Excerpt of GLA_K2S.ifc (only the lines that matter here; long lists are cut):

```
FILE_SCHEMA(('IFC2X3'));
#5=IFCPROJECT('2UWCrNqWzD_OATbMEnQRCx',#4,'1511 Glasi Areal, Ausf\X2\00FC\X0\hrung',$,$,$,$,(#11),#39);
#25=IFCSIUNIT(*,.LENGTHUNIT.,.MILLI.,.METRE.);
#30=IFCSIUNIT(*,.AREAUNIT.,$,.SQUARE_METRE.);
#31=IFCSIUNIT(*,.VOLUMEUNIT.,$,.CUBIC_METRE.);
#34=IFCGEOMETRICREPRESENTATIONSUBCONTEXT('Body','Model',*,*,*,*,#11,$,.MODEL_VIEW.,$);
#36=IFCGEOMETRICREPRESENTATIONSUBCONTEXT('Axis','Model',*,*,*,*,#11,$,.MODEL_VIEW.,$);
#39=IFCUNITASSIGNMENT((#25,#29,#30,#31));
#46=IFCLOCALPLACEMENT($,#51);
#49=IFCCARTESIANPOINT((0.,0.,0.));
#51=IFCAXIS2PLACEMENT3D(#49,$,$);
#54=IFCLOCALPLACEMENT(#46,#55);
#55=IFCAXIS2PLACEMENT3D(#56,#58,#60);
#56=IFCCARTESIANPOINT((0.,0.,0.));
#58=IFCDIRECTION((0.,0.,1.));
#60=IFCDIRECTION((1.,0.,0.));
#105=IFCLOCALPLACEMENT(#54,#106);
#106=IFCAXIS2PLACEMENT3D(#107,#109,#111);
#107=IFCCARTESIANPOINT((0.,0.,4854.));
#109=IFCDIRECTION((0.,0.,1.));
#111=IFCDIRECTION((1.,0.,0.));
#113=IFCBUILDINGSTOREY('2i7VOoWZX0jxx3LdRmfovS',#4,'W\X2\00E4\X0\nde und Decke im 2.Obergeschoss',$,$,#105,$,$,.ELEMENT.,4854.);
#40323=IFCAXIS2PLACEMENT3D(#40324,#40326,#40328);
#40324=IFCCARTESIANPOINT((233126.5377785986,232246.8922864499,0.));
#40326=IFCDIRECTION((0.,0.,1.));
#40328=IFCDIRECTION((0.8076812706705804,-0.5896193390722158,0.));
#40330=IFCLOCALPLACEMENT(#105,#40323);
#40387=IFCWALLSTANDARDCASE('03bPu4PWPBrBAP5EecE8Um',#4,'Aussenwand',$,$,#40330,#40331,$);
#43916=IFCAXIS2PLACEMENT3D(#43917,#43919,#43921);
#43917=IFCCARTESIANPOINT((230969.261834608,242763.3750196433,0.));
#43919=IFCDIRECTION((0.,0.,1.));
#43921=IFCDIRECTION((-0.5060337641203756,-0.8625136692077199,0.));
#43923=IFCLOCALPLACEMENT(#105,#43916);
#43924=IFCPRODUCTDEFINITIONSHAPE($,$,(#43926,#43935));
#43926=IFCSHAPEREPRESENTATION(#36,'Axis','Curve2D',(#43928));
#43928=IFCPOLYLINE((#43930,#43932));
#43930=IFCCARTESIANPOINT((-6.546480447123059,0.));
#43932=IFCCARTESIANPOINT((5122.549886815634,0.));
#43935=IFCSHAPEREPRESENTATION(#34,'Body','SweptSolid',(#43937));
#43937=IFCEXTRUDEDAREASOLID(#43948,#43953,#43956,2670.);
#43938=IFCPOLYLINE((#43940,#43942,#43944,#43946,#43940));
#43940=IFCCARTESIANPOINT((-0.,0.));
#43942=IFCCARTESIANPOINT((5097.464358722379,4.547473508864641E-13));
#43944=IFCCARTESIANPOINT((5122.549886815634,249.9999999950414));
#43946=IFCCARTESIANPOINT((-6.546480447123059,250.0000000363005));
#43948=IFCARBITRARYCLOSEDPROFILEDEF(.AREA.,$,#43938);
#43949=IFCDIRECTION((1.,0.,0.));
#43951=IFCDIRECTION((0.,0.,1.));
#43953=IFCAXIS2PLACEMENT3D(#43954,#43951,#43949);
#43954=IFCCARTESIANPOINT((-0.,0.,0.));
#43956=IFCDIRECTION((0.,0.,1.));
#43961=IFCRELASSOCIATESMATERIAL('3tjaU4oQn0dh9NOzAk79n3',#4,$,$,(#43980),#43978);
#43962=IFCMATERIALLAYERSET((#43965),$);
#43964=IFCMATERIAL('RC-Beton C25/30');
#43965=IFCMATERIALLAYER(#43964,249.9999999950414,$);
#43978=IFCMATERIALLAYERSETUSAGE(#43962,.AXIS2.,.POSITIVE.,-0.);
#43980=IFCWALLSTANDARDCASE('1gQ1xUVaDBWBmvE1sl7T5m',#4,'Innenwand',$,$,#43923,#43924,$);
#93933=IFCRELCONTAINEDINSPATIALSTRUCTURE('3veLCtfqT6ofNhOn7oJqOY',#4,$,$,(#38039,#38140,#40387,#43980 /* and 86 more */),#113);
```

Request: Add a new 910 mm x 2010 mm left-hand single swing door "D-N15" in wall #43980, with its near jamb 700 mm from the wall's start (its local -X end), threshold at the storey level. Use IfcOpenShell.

```python
import numpy as np
import ifcopenshell
import ifcopenshell.api.feature
import ifcopenshell.api.geometry
import ifcopenshell.api.root
import ifcopenshell.api.spatial
import ifcopenshell.api.type
import ifcopenshell.geom
import ifcopenshell.util.element
import ifcopenshell.util.placement
import ifcopenshell.util.representation
import ifcopenshell.util.shape
import ifcopenshell.util.unit

model = ifcopenshell.open("GLA_K2S.ifc")
unit_scale = ifcopenshell.util.unit.calculate_unit_scale(model)
settings = ifcopenshell.geom.settings()


def volume(element):
    """Net volume in cubic metres, openings subtracted."""
    shape = ifcopenshell.geom.create_shape(settings, element)
    return ifcopenshell.util.shape.get_volume(shape.geometry)


wall = model.by_id(43980)
storey = ifcopenshell.util.element.get_container(wall, ifc_class="IfcBuildingStorey")
context = ifcopenshell.util.representation.get_context(model, "Model", "Body", "MODEL_VIEW")
before = volume(wall)

width, height, from_end, sill = 0.91, 2.01, 0.7, 0.0  # metres

# The wall runs along its own X axis, and the end named is its -X end.
wall_shape = ifcopenshell.geom.create_shape(settings, wall)
x, y, z = ifcopenshell.util.shape.get_vertices(wall_shape.geometry).T
start = x.min() + from_end
face, thickness = float(y.min()), float(y.max() - y.min())
wall_matrix = ifcopenshell.util.placement.get_local_placement(wall.ObjectPlacement)
level = ifcopenshell.util.placement.get_local_placement(storey.ObjectPlacement)[2, 3]


def in_wall(x, y):
    """Placement at x, y metres in the wall's axes, at sill height."""
    matrix = wall_matrix.copy()
    matrix[:, 3] = wall_matrix @ np.array([x / unit_scale, y / unit_scale, 0.0, 1.0])
    matrix[2, 3] = level + sill / unit_scale
    return matrix


# Opening: a box that overshoots both wall faces by 50 mm.
opening = ifcopenshell.api.root.create_entity(model, ifc_class="IfcOpeningElement")
box = ifcopenshell.api.geometry.add_wall_representation(
    model, context=context, length=width, height=height, thickness=thickness + 0.1
)
ifcopenshell.api.geometry.assign_representation(model, product=opening, representation=box)
ifcopenshell.api.geometry.edit_object_placement(model, product=opening, matrix=in_wall(start, face - 0.05), is_si=False)
ifcopenshell.api.feature.add_feature(model, feature=opening, element=wall)

door = ifcopenshell.api.root.create_entity(model, ifc_class="IfcDoor", name="D-N15")
door.OverallWidth, door.OverallHeight = width / unit_scale, height / unit_scale
body = ifcopenshell.api.geometry.add_door_representation(
    model,
    context=context,
    overall_width=door.OverallWidth,
    overall_height=door.OverallHeight,
    operation_type="SINGLE_SWING_LEFT",
    lining_properties={"LiningDepth": thickness / unit_scale, "ThresholdDepth": thickness / unit_scale},
)
ifcopenshell.api.geometry.assign_representation(model, product=door, representation=body)
ifcopenshell.api.spatial.assign_container(model, products=[door], relating_structure=storey)
fills = ifcopenshell.api.feature.add_filling(model, opening=opening, element=door)
fills.OwnerHistory = door.OwnerHistory  # required in IFC2X3

# IFC2X3 keeps the operation on the door style.
style = ifcopenshell.api.root.create_entity(model, ifc_class="IfcDoorStyle", name="D-N15")
style.OperationType, style.ConstructionType = "SINGLE_SWING_LEFT", "NOTDEFINED"
style.ParameterTakesPrecedence = style.Sizeable = False
ifcopenshell.api.type.assign_type(model, related_objects=[door], relating_type=style)

# The lining spans the wall, so the door starts at the wall face.
ifcopenshell.api.geometry.edit_object_placement(model, product=door, matrix=in_wall(start, face), is_si=False)

after = volume(wall)

print(f"wall volume {before:.3f} -> {after:.3f} m3")

model.write("GLA_K2S_edited.ifc")
```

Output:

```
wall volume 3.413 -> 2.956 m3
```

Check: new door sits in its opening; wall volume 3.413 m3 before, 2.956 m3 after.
